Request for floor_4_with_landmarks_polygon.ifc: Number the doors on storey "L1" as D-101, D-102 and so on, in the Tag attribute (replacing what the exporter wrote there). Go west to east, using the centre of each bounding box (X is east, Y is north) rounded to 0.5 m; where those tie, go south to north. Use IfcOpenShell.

First a look at what the model holds.

```python
import ifcopenshell
import ifcopenshell.util.element
import ifcopenshell.util.placement

model = ifcopenshell.open("floor_4_with_landmarks_polygon.ifc")
print(model.schema)
storey = next(s for s in model.by_type("IfcBuildingStorey") if s.Name == "L1")
doors = [e for e in ifcopenshell.util.element.get_decomposition(storey) if e.is_a("IfcDoor")]
for e in sorted(doors, key=lambda e: e.id()):
    origin = ifcopenshell.util.placement.get_local_placement(e.ObjectPlacement)[:3, 3]
    print(e.id(), e.Tag, e.Name, origin.round(2) + 0.0, sep=" | ")
```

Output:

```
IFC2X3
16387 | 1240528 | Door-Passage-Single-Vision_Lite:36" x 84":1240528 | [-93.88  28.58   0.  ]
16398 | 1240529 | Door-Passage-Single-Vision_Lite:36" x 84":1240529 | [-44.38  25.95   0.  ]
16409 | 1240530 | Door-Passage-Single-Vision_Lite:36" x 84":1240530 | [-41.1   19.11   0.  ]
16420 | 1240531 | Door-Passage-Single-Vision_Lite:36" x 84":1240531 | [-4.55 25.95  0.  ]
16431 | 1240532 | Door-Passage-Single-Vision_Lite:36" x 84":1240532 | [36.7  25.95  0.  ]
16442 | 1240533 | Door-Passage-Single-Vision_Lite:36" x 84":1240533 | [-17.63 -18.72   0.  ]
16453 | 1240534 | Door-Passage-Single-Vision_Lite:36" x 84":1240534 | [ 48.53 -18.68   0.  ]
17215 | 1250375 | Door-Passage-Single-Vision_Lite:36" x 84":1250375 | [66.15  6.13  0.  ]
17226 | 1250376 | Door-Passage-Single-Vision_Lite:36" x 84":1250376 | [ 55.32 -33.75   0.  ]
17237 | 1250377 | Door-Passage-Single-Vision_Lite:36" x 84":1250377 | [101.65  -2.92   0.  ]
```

```python
import ifcopenshell
import ifcopenshell.geom
import ifcopenshell.util.element
import ifcopenshell.util.shape

model = ifcopenshell.open("floor_4_with_landmarks_polygon.ifc")
settings = ifcopenshell.geom.settings()
settings.set("use-world-coords", True)


def centre(element):
    shape = ifcopenshell.geom.create_shape(settings, element)
    return ifcopenshell.util.shape.get_bbox_centroid(shape.geometry)


storey = next(s for s in model.by_type("IfcBuildingStorey") if s.Name == "L1")
doors = [e for e in ifcopenshell.util.element.get_decomposition(storey) if e.is_a("IfcDoor")]

# Insertion points can sit at a corner or the storey origin, so sort by the geometry (in metres).
centres = {e: centre(e) for e in doors}
doors.sort(key=lambda e: (round(centres[e][0] / 0.5), centres[e][1]))

for i, e in enumerate(doors, start=1):
    number = f"D-1{i:02d}"
    e.Tag = number
    print(e.id(), number)

model.write("floor_4_with_landmarks_polygon_updated.ifc")
```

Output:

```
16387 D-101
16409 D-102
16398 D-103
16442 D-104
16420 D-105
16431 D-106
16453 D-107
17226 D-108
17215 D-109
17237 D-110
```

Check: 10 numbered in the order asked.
